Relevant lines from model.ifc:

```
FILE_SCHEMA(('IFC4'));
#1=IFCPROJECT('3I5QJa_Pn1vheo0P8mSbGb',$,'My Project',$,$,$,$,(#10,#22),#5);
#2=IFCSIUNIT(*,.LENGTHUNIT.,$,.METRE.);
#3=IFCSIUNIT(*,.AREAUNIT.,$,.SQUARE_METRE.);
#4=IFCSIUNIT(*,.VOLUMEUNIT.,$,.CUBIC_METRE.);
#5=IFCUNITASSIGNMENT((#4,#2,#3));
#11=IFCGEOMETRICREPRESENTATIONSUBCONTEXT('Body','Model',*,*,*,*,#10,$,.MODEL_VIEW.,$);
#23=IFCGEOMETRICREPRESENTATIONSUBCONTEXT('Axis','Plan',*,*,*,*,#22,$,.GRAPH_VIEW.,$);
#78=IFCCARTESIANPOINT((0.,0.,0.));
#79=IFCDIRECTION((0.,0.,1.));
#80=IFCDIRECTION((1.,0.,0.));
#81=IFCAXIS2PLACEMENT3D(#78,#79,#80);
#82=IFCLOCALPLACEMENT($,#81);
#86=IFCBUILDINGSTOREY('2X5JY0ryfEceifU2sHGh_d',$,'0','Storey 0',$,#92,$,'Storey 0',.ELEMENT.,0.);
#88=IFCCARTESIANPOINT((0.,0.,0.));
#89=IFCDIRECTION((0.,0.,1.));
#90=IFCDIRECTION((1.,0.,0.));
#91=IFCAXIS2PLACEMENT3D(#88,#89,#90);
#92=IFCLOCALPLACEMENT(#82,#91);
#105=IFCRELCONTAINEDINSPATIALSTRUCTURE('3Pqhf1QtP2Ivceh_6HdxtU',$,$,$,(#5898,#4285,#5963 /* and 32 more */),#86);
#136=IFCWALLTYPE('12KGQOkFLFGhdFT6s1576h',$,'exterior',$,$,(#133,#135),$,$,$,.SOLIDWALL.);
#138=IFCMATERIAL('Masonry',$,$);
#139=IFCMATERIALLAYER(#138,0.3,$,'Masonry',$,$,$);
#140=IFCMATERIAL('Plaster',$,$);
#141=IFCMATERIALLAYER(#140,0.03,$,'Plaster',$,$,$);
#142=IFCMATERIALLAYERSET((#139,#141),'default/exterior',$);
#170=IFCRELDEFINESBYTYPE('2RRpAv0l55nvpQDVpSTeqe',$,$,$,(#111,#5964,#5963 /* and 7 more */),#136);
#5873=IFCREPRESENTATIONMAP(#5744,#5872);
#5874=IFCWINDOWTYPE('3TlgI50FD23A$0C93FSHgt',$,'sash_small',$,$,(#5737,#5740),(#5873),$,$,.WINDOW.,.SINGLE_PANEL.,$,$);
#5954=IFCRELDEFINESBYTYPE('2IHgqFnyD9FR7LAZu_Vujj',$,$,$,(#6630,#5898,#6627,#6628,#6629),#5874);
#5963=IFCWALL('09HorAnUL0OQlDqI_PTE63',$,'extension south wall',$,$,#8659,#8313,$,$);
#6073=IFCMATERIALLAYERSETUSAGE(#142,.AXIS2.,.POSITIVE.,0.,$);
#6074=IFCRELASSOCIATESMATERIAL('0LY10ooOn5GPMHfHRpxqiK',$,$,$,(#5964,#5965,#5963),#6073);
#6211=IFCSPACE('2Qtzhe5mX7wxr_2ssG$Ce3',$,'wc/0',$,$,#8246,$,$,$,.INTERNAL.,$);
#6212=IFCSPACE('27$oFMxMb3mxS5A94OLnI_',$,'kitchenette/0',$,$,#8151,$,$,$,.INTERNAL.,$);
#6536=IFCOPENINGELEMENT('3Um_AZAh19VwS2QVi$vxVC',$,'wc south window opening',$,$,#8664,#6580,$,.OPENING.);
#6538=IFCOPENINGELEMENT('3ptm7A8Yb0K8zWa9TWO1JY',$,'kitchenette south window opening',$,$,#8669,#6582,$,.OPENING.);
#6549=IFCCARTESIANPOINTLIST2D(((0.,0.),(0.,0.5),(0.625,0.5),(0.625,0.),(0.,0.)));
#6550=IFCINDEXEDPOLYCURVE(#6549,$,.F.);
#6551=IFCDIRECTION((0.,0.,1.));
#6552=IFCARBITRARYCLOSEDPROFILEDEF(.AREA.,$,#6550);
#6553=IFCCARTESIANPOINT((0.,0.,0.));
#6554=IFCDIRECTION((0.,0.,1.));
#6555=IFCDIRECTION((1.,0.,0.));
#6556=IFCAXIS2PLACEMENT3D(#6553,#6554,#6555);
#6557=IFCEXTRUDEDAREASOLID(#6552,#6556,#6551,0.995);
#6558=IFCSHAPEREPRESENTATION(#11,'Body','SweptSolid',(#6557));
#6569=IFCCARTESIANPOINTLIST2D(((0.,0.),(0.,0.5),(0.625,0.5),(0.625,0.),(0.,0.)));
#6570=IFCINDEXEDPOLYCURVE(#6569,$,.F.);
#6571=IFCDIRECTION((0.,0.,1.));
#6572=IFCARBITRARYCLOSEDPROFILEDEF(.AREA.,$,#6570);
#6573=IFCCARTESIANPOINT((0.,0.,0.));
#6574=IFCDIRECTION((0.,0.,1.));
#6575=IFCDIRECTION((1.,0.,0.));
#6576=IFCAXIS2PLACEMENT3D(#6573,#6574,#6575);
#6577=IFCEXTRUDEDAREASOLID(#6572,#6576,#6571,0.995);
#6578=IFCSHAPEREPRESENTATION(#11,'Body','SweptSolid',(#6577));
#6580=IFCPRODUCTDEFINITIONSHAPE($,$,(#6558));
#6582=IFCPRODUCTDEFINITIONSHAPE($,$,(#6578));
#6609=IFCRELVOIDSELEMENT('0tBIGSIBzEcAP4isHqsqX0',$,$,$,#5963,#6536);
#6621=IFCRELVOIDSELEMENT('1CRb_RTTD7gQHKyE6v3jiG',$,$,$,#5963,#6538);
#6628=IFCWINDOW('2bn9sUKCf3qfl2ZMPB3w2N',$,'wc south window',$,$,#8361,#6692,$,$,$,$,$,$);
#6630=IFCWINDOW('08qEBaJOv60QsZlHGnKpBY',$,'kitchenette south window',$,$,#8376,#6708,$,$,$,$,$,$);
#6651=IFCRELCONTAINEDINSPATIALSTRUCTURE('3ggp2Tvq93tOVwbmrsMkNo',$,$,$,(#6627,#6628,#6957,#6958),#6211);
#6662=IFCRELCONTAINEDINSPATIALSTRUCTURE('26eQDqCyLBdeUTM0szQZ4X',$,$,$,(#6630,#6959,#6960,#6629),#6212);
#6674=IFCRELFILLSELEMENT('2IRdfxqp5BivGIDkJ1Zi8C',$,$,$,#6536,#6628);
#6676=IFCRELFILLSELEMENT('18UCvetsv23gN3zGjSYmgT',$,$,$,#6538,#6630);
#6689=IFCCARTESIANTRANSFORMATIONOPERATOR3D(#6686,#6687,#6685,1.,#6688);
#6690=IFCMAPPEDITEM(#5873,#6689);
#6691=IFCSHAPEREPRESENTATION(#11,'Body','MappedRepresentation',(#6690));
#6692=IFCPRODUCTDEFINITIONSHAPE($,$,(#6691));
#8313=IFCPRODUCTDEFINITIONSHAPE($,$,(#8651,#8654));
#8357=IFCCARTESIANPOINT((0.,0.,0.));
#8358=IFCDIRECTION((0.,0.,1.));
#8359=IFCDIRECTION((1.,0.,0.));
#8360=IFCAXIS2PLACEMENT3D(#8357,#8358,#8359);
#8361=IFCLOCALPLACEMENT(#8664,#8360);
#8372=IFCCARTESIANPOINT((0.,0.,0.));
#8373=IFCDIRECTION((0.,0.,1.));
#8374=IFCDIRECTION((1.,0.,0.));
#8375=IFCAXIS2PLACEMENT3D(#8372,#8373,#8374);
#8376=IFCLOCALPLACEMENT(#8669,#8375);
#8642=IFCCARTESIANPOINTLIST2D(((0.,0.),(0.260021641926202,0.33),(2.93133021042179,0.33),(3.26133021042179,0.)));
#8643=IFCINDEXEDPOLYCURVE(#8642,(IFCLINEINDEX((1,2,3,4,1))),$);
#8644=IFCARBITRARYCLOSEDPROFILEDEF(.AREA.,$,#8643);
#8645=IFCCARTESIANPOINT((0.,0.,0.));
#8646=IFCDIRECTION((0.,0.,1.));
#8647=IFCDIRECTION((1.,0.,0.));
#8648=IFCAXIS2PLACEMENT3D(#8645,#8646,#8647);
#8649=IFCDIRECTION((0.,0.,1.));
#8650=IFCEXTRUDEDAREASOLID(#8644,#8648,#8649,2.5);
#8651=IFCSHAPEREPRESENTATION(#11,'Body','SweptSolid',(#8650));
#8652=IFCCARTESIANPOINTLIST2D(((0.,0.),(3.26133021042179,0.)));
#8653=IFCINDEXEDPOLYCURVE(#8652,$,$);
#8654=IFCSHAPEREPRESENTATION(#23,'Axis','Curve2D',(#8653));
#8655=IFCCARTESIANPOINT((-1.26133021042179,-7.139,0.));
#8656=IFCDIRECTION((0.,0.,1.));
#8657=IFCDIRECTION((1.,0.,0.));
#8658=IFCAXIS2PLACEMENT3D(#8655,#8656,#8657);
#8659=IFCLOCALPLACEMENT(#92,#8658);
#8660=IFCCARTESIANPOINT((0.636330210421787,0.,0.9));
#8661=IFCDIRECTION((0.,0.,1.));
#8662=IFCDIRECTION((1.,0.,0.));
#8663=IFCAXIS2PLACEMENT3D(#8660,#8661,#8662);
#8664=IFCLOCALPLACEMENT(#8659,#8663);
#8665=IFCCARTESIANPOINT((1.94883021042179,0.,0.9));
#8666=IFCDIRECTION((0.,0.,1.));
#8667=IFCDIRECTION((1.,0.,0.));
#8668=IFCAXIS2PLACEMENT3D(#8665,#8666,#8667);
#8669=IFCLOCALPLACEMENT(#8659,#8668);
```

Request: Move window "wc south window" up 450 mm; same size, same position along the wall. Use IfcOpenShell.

```python
import numpy as np
import ifcopenshell
import ifcopenshell.api.geometry
import ifcopenshell.util.placement
import ifcopenshell.util.unit

model = ifcopenshell.open("model.ifc")
unit_scale = ifcopenshell.util.unit.calculate_unit_scale(model)

window = model.by_guid("2bn9sUKCf3qfl2ZMPB3w2N")
opening = window.FillsVoids[0].RelatingOpeningElement
dz = 0.45 / unit_scale

shift = np.array([0.0, 0.0, dz])
# The window is placed relative to its opening, so it follows when the opening moves.
matrix = ifcopenshell.util.placement.get_local_placement(opening.ObjectPlacement)
matrix[:3, 3] += shift
ifcopenshell.api.geometry.edit_object_placement(
    model, product=opening, matrix=matrix, is_si=False, should_transform_children=True
)

print(f"moved by {dz * unit_scale:+.3f} m")

model.write("model_edited.ifc")
```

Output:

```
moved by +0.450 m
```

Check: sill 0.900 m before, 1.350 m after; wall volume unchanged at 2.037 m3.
